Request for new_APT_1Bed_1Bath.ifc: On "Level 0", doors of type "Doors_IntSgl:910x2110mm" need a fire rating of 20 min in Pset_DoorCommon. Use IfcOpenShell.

First a look at what the model holds.

```python
import ifcopenshell
import ifcopenshell.util.element

model = ifcopenshell.open("new_APT_1Bed_1Bath.ifc")
print(model.schema)
storey = next(s for s in model.by_type("IfcBuildingStorey") if s.Name == "Level 0")
doors = [e for e in ifcopenshell.util.element.get_decomposition(storey) if e.is_a("IfcDoor")]
seen = {}
for e in doors:
    element_type = ifcopenshell.util.element.get_type(e)
    key = (element_type.Name if element_type != e and element_type else None, ifcopenshell.util.element.get_pset(e, "Pset_DoorCommon", "FireRating"))
    seen[key] = seen.get(key, 0) + 1
for (name, value), count in sorted(seen.items(), key=str):
    print(count, "x", name, "|", value)
```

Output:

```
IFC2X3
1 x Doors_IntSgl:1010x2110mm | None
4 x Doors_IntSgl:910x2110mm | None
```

```python
import ifcopenshell
import ifcopenshell.api.pset
import ifcopenshell.util.element

model = ifcopenshell.open("new_APT_1Bed_1Bath.ifc")

storey = next(s for s in model.by_type("IfcBuildingStorey") if s.Name == "Level 0")
doors = [e for e in ifcopenshell.util.element.get_decomposition(storey) if e.is_a("IfcDoor")]

count = 0
for e in doors:
    element_type = ifcopenshell.util.element.get_type(e)
    if element_type in (None, e) or element_type.Name != "Doors_IntSgl:910x2110mm":
        continue
    # add_pset returns the element's existing set when there is one.
    pset = ifcopenshell.api.pset.add_pset(model, product=e, name="Pset_DoorCommon")
    ifcopenshell.api.pset.edit_pset(model, pset=pset, properties={"FireRating": "20 min"})
    count += 1

print(count, "doors updated")

model.write("new_APT_1Bed_1Bath_v2.ifc")
```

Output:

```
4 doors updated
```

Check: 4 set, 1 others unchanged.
